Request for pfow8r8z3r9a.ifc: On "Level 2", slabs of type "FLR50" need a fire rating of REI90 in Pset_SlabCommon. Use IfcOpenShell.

First a look at what the model holds.

```python
import ifcopenshell
import ifcopenshell.util.element

model = ifcopenshell.open("pfow8r8z3r9a.ifc")
print(model.schema)
storey = next(s for s in model.by_type("IfcBuildingStorey") if s.Name == "Level 2")
slabs = [e for e in ifcopenshell.util.element.get_decomposition(storey) if e.is_a("IfcSlab")]
seen = {}
for e in slabs:
    element_type = ifcopenshell.util.element.get_type(e)
    key = (element_type.Name if element_type != e and element_type else None, ifcopenshell.util.element.get_pset(e, "Pset_SlabCommon", "FireRating"))
    seen[key] = seen.get(key, 0) + 1
for (name, value), count in sorted(seen.items(), key=str):
    print(count, "x", name, "|", value)
```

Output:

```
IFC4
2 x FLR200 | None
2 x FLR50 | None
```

```python
import ifcopenshell
import ifcopenshell.api.pset
import ifcopenshell.util.element

model = ifcopenshell.open("pfow8r8z3r9a.ifc")

storey = next(s for s in model.by_type("IfcBuildingStorey") if s.Name == "Level 2")
slabs = [e for e in ifcopenshell.util.element.get_decomposition(storey) if e.is_a("IfcSlab")]

count = 0
for e in slabs:
    element_type = ifcopenshell.util.element.get_type(e)
    if element_type in (None, e) or element_type.Name != "FLR50":
        continue
    # add_pset returns the element's existing set when there is one.
    pset = ifcopenshell.api.pset.add_pset(model, product=e, name="Pset_SlabCommon")
    ifcopenshell.api.pset.edit_pset(model, pset=pset, properties={"FireRating": "REI90"})
    count += 1

print(count, "slabs updated")

model.write("pfow8r8z3r9a_edited.ifc")
```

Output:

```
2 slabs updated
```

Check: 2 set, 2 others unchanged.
